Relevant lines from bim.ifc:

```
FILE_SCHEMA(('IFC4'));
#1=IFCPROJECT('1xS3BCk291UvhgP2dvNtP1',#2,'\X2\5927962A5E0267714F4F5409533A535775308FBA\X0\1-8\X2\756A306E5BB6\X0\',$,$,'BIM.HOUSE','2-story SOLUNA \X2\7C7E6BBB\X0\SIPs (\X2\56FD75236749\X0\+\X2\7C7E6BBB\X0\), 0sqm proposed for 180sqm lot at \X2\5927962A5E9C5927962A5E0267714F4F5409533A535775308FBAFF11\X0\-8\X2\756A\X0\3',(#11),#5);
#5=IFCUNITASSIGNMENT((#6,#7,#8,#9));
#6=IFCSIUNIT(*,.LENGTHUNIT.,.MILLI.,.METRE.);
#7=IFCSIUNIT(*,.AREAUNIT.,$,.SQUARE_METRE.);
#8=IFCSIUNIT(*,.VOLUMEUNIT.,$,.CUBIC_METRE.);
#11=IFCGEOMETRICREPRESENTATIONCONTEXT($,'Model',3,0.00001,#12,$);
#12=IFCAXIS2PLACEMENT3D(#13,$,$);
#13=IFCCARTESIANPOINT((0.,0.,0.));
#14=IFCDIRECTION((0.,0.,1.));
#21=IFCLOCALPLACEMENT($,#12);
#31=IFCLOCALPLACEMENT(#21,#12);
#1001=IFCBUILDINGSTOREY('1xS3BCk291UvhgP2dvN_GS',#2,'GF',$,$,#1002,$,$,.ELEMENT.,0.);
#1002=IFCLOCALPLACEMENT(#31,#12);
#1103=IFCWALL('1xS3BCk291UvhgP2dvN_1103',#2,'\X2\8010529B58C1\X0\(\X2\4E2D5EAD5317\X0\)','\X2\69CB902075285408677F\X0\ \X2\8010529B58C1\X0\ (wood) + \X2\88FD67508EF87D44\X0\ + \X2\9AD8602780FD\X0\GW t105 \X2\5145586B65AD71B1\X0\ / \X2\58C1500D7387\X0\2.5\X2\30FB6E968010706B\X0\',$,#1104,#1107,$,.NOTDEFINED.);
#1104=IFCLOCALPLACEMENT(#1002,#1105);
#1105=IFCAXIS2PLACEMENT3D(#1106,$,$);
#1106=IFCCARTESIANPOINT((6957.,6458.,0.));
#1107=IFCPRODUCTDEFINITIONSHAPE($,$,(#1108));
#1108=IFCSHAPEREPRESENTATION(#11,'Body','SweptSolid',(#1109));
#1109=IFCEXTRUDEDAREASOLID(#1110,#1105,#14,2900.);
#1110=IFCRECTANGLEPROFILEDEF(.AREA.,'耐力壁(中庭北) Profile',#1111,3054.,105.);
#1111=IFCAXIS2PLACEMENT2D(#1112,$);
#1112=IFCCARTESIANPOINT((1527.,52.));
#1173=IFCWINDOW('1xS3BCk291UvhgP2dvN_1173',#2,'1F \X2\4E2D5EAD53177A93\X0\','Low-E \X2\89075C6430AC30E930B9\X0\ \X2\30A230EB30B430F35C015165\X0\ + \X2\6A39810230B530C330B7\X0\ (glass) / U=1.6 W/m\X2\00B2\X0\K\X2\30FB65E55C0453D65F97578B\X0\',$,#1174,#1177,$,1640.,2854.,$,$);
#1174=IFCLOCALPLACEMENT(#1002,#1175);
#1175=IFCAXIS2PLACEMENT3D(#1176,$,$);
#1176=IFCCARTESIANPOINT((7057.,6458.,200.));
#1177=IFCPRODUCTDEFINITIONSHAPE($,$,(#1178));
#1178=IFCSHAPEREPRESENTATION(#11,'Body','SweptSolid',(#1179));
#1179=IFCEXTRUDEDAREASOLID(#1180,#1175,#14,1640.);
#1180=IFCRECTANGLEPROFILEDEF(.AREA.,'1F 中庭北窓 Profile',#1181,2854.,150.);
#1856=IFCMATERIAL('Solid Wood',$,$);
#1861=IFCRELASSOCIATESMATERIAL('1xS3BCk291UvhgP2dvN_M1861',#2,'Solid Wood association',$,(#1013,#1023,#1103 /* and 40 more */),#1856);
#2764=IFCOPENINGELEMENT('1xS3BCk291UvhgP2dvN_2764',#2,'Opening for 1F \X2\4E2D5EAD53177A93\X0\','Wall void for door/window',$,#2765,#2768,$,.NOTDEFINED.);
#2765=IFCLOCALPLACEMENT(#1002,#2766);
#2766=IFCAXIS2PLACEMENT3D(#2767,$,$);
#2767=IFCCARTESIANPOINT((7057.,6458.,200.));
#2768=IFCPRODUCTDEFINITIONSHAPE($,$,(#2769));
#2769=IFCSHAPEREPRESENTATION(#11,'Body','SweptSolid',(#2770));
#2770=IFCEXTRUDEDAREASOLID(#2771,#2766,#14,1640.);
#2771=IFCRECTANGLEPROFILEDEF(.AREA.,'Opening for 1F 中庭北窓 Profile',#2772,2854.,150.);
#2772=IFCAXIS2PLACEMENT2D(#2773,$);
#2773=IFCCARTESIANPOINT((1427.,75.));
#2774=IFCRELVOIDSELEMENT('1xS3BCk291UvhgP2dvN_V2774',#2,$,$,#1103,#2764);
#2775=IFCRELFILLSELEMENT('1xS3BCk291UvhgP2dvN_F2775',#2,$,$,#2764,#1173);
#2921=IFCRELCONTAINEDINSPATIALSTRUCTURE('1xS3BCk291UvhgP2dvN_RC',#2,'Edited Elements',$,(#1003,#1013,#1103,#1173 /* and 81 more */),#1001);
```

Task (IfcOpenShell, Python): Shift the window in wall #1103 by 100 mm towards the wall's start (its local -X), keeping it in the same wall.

```python
import ifcopenshell
import ifcopenshell.api.geometry
import ifcopenshell.util.placement

model = ifcopenshell.open("bim.ifc")

window = model.by_guid("1xS3BCk291UvhgP2dvN_1173")
opening = window.FillsVoids[0].RelatingOpeningElement
wall = opening.VoidsElements[0].RelatingBuildingElement

wall_matrix = ifcopenshell.util.placement.get_local_placement(wall.ObjectPlacement)
shift = wall_matrix[:3, 0] * -100.0
before = ifcopenshell.util.placement.get_local_placement(window.ObjectPlacement)[:3, 3].copy()

# The window is not placed relative to its opening, so move both.
for product in (opening, window):
    matrix = ifcopenshell.util.placement.get_local_placement(product.ObjectPlacement)
    matrix[:3, 3] += shift
    ifcopenshell.api.geometry.edit_object_placement(model, product=product, matrix=matrix, is_si=False)

after = ifcopenshell.util.placement.get_local_placement(window.ObjectPlacement)[:3, 3]
print("window moved by", (after - before).round(3) + 0.0)

model.write("bim-out.ifc")
```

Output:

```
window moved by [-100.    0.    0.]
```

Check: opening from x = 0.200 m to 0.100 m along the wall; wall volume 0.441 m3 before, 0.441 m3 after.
